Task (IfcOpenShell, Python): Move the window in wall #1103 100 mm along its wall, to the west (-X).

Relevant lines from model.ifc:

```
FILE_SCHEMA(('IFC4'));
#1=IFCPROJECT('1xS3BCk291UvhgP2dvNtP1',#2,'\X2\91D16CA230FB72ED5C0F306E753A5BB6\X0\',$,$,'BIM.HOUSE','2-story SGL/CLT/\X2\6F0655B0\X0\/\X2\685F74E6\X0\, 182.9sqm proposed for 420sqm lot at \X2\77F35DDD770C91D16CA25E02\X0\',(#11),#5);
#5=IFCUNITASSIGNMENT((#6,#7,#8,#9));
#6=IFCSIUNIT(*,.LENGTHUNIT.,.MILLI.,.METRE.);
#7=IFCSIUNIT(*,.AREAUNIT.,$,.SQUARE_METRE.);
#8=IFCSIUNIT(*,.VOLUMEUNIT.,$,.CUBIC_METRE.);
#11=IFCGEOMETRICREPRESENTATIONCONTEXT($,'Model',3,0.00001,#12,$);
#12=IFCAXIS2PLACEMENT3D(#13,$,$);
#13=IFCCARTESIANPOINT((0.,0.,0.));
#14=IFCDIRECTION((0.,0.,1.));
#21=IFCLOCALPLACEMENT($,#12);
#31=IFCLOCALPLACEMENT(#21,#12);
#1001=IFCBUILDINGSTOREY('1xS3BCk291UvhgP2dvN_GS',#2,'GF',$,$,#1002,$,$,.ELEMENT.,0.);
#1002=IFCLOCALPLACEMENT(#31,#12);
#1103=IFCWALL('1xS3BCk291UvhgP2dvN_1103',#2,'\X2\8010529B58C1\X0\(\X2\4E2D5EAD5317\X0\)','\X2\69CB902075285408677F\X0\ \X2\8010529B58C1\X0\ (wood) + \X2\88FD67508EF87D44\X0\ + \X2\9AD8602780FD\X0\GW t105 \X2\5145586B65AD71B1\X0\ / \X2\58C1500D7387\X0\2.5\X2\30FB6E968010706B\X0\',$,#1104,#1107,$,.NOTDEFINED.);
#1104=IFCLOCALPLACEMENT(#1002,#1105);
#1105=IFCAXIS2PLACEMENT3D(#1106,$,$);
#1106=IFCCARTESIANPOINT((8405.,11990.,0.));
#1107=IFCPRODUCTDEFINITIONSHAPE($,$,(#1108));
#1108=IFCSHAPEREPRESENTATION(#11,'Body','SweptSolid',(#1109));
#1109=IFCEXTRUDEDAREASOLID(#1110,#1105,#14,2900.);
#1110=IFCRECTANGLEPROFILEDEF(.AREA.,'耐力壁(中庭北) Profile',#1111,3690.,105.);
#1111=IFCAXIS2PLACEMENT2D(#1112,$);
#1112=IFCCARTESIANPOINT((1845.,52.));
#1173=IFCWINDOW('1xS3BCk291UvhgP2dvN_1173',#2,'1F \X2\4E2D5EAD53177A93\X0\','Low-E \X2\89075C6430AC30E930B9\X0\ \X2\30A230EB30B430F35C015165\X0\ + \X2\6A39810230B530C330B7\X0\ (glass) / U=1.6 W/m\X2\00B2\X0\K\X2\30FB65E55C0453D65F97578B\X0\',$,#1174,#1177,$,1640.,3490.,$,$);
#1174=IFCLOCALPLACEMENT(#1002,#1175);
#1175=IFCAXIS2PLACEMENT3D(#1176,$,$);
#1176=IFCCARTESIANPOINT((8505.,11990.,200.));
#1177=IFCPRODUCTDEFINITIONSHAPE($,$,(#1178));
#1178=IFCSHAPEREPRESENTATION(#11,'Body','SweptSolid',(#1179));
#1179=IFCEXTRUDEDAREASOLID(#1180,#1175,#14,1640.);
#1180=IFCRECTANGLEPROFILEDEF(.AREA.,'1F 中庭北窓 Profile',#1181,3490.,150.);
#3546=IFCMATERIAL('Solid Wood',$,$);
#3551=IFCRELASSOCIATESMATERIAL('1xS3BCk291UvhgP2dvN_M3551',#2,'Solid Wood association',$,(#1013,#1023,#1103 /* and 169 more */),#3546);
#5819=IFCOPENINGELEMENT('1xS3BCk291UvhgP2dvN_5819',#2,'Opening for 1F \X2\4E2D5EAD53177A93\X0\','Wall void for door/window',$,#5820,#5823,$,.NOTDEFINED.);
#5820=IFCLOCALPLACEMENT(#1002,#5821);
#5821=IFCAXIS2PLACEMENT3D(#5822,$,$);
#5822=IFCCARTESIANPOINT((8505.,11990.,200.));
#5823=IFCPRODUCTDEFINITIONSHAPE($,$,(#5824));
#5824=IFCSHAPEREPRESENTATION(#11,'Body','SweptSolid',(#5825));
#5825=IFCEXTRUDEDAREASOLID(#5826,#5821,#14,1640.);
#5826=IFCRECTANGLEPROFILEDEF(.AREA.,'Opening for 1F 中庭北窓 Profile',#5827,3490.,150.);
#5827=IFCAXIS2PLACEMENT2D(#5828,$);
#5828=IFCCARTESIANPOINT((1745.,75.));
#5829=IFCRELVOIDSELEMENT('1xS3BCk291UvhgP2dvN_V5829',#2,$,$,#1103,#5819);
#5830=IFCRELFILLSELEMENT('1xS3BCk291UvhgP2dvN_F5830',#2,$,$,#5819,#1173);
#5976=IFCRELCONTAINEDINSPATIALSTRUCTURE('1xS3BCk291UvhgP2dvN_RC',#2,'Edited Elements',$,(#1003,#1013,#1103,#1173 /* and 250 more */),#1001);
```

```python
import ifcopenshell
import ifcopenshell.api.geometry
import ifcopenshell.util.placement
import ifcopenshell.util.unit

model = ifcopenshell.open("model.ifc")
unit_scale = ifcopenshell.util.unit.calculate_unit_scale(model)

window = model.by_id(1173)
opening = window.FillsVoids[0].RelatingOpeningElement
wall = opening.VoidsElements[0].RelatingBuildingElement

wall_matrix = ifcopenshell.util.placement.get_local_placement(wall.ObjectPlacement)
shift = wall_matrix[:3, 0] * -0.1 / unit_scale
before = ifcopenshell.util.placement.get_local_placement(window.ObjectPlacement)[:3, 3].copy()

# The window is not placed relative to its opening, so move both.
for product in (opening, window):
    matrix = ifcopenshell.util.placement.get_local_placement(product.ObjectPlacement)
    matrix[:3, 3] += shift
    ifcopenshell.api.geometry.edit_object_placement(model, product=product, matrix=matrix, is_si=False)

after = ifcopenshell.util.placement.get_local_placement(window.ObjectPlacement)[:3, 3]
print("window moved by", (after - before).round(3) + 0.0)

model.write("model_updated.ifc")
```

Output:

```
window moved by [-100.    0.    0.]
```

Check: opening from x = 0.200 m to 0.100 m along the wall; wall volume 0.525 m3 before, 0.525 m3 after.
